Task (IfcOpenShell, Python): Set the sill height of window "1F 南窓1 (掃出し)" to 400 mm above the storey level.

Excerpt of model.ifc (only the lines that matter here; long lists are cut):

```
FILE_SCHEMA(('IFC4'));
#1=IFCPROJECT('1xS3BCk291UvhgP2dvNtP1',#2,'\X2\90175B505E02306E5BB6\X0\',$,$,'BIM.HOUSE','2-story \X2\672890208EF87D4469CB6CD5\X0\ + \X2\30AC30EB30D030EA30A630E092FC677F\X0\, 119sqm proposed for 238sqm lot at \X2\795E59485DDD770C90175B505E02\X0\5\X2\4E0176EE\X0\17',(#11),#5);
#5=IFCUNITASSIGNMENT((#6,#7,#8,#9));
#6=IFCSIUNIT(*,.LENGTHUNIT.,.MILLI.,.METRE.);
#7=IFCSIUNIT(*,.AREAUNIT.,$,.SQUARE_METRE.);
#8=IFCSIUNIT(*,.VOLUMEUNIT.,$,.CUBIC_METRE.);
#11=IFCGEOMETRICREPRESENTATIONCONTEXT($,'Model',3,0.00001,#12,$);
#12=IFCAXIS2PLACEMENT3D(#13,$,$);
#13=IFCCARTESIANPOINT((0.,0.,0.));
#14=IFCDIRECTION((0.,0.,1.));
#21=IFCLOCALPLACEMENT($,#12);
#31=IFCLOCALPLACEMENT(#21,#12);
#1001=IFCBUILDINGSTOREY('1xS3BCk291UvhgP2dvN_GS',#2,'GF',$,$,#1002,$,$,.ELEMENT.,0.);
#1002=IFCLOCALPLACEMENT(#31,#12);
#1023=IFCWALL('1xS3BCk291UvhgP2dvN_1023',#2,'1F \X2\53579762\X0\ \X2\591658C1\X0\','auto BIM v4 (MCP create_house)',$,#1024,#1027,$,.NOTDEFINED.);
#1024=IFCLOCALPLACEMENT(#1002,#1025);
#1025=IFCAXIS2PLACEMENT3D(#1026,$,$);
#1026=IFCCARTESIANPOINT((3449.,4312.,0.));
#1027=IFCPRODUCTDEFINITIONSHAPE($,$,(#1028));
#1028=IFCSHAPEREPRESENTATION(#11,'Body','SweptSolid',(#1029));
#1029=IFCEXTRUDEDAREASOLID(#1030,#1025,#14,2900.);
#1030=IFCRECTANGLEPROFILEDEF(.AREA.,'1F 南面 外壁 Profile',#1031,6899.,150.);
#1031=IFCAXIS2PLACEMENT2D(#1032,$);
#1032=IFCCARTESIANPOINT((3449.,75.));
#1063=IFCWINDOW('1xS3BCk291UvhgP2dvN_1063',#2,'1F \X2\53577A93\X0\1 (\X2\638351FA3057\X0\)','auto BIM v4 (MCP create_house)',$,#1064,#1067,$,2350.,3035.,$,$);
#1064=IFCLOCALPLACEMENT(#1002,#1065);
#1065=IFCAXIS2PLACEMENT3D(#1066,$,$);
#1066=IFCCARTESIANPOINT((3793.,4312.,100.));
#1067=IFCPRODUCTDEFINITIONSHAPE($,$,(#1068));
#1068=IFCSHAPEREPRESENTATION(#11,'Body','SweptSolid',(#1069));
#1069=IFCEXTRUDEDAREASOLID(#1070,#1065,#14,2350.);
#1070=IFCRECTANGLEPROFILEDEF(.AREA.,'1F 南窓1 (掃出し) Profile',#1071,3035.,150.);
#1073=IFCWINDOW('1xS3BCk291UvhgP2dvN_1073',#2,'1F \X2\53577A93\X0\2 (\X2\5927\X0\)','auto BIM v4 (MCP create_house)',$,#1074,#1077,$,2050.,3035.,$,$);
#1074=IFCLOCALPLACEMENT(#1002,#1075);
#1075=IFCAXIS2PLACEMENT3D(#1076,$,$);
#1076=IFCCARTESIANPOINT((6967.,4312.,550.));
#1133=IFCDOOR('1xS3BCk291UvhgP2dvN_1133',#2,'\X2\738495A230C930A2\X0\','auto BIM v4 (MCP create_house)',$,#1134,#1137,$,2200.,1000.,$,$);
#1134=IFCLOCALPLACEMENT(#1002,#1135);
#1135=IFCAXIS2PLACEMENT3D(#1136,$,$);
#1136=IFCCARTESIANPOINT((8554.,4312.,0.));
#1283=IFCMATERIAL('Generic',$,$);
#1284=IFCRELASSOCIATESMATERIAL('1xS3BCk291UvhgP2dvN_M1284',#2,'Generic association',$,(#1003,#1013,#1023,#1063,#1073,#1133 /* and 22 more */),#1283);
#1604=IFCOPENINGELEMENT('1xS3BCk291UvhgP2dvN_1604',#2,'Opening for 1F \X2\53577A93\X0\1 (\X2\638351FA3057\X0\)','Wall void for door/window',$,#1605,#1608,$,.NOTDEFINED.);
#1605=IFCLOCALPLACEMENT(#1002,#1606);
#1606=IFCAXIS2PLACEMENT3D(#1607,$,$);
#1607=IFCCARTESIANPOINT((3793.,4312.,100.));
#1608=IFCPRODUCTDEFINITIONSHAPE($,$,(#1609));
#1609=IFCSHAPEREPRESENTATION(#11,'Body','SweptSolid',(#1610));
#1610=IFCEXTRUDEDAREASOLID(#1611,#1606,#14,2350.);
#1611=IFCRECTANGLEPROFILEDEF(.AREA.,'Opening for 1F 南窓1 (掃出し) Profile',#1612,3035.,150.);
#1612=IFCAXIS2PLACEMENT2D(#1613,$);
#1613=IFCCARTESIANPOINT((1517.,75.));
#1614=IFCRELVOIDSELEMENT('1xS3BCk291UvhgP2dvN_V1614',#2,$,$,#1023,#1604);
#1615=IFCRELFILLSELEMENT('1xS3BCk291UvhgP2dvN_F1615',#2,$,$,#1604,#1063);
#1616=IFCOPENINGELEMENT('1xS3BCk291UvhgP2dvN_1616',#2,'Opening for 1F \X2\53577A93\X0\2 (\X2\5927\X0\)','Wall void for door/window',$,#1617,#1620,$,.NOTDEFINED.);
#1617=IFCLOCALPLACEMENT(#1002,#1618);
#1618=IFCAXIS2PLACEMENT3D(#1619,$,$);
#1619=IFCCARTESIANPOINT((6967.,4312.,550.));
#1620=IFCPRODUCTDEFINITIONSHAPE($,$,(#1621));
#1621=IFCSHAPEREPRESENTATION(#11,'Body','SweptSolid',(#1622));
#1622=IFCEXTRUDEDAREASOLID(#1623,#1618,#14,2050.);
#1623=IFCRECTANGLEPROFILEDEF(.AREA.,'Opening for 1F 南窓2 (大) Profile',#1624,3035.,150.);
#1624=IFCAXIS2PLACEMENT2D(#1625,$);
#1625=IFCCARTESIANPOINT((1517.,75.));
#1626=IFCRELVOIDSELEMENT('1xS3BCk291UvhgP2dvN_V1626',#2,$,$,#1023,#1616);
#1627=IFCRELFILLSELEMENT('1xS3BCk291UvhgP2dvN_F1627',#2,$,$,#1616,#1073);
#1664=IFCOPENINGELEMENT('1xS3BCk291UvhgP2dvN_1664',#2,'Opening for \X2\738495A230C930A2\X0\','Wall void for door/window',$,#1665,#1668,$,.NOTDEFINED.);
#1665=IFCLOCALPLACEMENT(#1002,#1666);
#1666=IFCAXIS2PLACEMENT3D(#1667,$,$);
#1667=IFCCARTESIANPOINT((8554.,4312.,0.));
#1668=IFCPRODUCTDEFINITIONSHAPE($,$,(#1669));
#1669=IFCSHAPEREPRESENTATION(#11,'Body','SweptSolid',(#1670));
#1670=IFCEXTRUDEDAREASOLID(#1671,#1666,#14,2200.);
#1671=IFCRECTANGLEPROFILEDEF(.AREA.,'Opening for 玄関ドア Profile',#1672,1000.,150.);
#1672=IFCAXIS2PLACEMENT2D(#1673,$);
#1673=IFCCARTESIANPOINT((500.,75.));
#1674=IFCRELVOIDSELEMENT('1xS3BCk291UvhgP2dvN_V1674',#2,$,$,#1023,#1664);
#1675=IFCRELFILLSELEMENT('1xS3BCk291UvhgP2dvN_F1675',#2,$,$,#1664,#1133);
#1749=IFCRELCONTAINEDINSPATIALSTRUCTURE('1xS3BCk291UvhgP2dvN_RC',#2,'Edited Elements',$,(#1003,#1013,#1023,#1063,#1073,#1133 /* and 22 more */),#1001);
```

```python
import numpy as np
import ifcopenshell
import ifcopenshell.api.geometry
import ifcopenshell.geom
import ifcopenshell.util.element
import ifcopenshell.util.placement
import ifcopenshell.util.shape
import ifcopenshell.util.unit

model = ifcopenshell.open("model.ifc")
unit_scale = ifcopenshell.util.unit.calculate_unit_scale(model)

window = model.by_guid("1xS3BCk291UvhgP2dvN_1063")
opening = window.FillsVoids[0].RelatingOpeningElement
storey = ifcopenshell.util.element.get_container(window, ifc_class="IfcBuildingStorey")
level = ifcopenshell.util.placement.get_local_placement(storey.ObjectPlacement)[2, 3]

# The opening's origin need not be at the sill, so measure its lowest point.
shape = ifcopenshell.geom.create_shape(ifcopenshell.geom.settings(), opening)
bottom = ifcopenshell.util.shape.get_shape_bottom_elevation(shape, shape.geometry) / unit_scale
dz = level + 400.0 - bottom

shift = np.array([0.0, 0.0, dz])
# The window is not placed relative to its opening, so move both.
for product in (opening, window):
    matrix = ifcopenshell.util.placement.get_local_placement(product.ObjectPlacement)
    matrix[:3, 3] += shift
    ifcopenshell.api.geometry.edit_object_placement(model, product=product, matrix=matrix, is_si=False)

print(f"moved by {dz * unit_scale:+.3f} m")

model.write("model-out.ifc")
```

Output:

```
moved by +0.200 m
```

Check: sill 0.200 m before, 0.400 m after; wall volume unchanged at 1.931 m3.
